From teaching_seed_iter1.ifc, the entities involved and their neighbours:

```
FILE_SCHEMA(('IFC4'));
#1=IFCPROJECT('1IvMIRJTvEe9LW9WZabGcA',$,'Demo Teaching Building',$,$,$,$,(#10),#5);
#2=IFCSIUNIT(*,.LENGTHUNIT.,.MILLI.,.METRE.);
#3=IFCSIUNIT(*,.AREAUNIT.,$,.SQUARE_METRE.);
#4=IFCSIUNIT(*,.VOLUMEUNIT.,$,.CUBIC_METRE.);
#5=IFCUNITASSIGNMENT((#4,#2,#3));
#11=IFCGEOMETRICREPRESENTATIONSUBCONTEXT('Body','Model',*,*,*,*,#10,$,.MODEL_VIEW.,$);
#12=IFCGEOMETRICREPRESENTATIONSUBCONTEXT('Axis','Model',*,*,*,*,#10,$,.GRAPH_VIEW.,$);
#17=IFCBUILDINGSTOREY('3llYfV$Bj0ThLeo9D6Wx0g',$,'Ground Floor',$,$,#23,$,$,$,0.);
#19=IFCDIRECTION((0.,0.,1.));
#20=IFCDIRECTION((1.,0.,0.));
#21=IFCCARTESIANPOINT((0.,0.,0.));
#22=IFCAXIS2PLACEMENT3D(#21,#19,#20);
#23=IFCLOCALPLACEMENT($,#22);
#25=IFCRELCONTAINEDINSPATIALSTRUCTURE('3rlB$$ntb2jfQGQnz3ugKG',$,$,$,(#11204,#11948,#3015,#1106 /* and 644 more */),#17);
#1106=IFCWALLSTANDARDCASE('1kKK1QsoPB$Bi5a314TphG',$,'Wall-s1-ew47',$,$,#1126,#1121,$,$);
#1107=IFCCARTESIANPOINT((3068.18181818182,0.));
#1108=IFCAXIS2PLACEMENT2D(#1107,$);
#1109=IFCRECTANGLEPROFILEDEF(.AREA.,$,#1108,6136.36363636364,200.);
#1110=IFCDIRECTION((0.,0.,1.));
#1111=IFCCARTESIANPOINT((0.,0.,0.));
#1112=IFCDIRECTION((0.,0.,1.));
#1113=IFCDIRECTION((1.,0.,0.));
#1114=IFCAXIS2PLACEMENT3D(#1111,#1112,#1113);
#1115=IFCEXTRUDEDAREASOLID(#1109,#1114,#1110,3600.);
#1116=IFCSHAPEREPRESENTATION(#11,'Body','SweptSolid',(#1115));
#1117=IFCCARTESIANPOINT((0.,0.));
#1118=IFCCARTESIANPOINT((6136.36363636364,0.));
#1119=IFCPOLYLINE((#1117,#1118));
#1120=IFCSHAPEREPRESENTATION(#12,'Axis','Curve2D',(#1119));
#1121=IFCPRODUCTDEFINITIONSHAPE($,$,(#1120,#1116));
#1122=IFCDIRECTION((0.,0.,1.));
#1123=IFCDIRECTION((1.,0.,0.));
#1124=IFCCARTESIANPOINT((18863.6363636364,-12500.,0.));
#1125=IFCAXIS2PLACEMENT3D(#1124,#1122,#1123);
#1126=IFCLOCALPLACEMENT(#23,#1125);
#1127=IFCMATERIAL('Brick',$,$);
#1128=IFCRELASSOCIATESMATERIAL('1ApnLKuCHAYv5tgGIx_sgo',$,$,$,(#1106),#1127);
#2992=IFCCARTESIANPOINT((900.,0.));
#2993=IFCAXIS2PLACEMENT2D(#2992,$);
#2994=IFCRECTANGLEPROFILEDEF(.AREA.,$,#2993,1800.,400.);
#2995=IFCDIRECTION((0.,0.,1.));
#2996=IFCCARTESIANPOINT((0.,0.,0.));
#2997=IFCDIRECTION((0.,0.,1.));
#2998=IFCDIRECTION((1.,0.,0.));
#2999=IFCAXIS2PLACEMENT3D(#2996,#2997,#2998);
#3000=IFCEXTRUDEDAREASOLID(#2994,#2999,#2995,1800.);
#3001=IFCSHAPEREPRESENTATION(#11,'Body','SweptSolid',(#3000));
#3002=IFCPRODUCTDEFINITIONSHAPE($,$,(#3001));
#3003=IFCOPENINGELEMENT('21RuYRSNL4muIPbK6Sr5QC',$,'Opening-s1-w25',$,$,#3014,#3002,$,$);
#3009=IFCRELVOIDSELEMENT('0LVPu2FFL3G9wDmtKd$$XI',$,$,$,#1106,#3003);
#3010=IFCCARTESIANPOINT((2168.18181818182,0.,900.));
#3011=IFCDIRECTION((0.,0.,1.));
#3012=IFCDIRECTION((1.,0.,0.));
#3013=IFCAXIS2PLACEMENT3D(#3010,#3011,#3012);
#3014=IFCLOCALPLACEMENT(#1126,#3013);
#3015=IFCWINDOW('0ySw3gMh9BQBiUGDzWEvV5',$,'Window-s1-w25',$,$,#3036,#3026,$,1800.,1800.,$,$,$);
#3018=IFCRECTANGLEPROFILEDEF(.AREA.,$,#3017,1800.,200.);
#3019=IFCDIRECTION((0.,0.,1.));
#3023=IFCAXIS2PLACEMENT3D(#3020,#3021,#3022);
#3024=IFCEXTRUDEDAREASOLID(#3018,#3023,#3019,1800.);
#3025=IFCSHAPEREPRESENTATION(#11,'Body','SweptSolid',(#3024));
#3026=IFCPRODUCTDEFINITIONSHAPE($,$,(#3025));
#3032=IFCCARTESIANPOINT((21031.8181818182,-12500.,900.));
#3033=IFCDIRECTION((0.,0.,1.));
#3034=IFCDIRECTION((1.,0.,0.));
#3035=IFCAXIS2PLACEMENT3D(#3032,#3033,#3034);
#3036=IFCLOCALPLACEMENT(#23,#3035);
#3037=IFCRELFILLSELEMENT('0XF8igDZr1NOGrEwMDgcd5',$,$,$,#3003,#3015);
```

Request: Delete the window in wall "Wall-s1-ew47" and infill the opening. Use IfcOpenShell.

```python
import ifcopenshell
import ifcopenshell.api.feature
import ifcopenshell.api.root
import ifcopenshell.geom
import ifcopenshell.util.shape

model = ifcopenshell.open("teaching_seed_iter1.ifc")
settings = ifcopenshell.geom.settings()


def volume(element):
    """Net volume in cubic metres, openings subtracted."""
    shape = ifcopenshell.geom.create_shape(settings, element)
    return ifcopenshell.util.shape.get_volume(shape.geometry)


window = model.by_guid("0ySw3gMh9BQBiUGDzWEvV5")
opening = window.FillsVoids[0].RelatingOpeningElement
wall = opening.VoidsElements[0].RelatingBuildingElement
before = volume(wall)

ifcopenshell.api.root.remove_product(model, product=window)
ifcopenshell.api.feature.remove_feature(model, feature=opening)

after = volume(wall)

print(f"wall volume {before:.3f} -> {after:.3f} m3")

model.write("teaching_seed_iter1-out.ifc")
```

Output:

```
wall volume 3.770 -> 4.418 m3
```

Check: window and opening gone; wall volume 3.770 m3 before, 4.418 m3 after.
